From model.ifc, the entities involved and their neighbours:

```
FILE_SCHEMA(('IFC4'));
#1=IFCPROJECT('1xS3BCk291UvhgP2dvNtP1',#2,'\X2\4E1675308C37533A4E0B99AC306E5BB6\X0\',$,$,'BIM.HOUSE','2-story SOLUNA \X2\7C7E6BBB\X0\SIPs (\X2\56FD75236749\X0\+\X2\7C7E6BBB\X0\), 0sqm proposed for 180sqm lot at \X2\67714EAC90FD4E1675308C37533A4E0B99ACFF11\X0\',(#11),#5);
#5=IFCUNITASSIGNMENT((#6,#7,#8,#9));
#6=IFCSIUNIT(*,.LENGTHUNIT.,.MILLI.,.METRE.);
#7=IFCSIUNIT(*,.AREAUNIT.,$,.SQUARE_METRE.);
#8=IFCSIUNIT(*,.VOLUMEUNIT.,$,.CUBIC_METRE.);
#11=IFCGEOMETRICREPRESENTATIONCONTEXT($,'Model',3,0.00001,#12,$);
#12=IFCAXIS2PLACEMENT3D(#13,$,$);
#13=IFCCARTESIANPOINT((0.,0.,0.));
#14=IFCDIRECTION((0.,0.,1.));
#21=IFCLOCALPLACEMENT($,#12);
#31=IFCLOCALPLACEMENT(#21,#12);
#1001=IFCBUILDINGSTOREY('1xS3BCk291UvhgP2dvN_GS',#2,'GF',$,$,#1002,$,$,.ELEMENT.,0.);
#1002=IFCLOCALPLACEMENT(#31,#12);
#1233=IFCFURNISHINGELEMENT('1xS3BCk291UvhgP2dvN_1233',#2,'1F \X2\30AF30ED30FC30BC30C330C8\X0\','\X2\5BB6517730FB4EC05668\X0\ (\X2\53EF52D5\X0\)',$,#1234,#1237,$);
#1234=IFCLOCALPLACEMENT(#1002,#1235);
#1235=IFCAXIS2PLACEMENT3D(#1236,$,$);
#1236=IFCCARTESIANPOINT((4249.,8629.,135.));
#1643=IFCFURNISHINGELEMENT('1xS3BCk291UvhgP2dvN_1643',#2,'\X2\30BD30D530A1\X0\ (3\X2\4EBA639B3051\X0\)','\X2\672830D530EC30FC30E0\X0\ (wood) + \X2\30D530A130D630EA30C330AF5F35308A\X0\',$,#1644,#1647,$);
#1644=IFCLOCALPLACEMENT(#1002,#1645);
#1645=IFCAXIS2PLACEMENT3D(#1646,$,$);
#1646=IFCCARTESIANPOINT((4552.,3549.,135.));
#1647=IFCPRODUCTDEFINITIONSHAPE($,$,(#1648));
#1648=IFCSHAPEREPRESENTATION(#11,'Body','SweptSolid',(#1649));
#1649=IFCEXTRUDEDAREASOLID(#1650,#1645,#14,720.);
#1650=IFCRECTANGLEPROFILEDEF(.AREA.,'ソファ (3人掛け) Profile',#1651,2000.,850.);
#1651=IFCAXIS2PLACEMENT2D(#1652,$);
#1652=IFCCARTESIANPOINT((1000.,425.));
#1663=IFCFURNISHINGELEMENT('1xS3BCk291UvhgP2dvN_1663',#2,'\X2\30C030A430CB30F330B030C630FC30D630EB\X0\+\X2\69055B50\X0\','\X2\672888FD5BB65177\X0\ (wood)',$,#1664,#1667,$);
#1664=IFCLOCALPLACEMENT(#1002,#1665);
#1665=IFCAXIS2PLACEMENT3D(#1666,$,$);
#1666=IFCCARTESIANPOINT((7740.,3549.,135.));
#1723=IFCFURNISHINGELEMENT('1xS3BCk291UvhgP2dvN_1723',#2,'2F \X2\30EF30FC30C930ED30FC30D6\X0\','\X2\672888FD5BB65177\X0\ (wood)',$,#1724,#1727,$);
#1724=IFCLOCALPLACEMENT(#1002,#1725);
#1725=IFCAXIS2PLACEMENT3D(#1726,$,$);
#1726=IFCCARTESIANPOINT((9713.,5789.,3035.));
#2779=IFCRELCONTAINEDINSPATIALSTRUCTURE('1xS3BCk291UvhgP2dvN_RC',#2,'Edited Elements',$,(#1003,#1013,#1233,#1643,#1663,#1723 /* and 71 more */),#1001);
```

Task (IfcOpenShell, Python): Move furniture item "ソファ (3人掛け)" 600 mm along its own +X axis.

```python
import ifcopenshell
import ifcopenshell.api.geometry
import ifcopenshell.util.placement
import ifcopenshell.util.unit

model = ifcopenshell.open("model.ifc")
unit_scale = ifcopenshell.util.unit.calculate_unit_scale(model)

item = model.by_id(1643)
matrix = ifcopenshell.util.placement.get_local_placement(item.ObjectPlacement)
matrix[:3, 3] += matrix[:3, 0] * 0.6 / unit_scale
ifcopenshell.api.geometry.edit_object_placement(model, product=item, matrix=matrix, is_si=False)

print(ifcopenshell.util.placement.get_local_placement(item.ObjectPlacement).round(3) + 0.0)

model.write("model_edited.ifc")
```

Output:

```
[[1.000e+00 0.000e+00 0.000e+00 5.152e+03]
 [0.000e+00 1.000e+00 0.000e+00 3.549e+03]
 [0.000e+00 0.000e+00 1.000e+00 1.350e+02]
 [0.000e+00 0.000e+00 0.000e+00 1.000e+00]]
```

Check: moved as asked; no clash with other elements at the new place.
